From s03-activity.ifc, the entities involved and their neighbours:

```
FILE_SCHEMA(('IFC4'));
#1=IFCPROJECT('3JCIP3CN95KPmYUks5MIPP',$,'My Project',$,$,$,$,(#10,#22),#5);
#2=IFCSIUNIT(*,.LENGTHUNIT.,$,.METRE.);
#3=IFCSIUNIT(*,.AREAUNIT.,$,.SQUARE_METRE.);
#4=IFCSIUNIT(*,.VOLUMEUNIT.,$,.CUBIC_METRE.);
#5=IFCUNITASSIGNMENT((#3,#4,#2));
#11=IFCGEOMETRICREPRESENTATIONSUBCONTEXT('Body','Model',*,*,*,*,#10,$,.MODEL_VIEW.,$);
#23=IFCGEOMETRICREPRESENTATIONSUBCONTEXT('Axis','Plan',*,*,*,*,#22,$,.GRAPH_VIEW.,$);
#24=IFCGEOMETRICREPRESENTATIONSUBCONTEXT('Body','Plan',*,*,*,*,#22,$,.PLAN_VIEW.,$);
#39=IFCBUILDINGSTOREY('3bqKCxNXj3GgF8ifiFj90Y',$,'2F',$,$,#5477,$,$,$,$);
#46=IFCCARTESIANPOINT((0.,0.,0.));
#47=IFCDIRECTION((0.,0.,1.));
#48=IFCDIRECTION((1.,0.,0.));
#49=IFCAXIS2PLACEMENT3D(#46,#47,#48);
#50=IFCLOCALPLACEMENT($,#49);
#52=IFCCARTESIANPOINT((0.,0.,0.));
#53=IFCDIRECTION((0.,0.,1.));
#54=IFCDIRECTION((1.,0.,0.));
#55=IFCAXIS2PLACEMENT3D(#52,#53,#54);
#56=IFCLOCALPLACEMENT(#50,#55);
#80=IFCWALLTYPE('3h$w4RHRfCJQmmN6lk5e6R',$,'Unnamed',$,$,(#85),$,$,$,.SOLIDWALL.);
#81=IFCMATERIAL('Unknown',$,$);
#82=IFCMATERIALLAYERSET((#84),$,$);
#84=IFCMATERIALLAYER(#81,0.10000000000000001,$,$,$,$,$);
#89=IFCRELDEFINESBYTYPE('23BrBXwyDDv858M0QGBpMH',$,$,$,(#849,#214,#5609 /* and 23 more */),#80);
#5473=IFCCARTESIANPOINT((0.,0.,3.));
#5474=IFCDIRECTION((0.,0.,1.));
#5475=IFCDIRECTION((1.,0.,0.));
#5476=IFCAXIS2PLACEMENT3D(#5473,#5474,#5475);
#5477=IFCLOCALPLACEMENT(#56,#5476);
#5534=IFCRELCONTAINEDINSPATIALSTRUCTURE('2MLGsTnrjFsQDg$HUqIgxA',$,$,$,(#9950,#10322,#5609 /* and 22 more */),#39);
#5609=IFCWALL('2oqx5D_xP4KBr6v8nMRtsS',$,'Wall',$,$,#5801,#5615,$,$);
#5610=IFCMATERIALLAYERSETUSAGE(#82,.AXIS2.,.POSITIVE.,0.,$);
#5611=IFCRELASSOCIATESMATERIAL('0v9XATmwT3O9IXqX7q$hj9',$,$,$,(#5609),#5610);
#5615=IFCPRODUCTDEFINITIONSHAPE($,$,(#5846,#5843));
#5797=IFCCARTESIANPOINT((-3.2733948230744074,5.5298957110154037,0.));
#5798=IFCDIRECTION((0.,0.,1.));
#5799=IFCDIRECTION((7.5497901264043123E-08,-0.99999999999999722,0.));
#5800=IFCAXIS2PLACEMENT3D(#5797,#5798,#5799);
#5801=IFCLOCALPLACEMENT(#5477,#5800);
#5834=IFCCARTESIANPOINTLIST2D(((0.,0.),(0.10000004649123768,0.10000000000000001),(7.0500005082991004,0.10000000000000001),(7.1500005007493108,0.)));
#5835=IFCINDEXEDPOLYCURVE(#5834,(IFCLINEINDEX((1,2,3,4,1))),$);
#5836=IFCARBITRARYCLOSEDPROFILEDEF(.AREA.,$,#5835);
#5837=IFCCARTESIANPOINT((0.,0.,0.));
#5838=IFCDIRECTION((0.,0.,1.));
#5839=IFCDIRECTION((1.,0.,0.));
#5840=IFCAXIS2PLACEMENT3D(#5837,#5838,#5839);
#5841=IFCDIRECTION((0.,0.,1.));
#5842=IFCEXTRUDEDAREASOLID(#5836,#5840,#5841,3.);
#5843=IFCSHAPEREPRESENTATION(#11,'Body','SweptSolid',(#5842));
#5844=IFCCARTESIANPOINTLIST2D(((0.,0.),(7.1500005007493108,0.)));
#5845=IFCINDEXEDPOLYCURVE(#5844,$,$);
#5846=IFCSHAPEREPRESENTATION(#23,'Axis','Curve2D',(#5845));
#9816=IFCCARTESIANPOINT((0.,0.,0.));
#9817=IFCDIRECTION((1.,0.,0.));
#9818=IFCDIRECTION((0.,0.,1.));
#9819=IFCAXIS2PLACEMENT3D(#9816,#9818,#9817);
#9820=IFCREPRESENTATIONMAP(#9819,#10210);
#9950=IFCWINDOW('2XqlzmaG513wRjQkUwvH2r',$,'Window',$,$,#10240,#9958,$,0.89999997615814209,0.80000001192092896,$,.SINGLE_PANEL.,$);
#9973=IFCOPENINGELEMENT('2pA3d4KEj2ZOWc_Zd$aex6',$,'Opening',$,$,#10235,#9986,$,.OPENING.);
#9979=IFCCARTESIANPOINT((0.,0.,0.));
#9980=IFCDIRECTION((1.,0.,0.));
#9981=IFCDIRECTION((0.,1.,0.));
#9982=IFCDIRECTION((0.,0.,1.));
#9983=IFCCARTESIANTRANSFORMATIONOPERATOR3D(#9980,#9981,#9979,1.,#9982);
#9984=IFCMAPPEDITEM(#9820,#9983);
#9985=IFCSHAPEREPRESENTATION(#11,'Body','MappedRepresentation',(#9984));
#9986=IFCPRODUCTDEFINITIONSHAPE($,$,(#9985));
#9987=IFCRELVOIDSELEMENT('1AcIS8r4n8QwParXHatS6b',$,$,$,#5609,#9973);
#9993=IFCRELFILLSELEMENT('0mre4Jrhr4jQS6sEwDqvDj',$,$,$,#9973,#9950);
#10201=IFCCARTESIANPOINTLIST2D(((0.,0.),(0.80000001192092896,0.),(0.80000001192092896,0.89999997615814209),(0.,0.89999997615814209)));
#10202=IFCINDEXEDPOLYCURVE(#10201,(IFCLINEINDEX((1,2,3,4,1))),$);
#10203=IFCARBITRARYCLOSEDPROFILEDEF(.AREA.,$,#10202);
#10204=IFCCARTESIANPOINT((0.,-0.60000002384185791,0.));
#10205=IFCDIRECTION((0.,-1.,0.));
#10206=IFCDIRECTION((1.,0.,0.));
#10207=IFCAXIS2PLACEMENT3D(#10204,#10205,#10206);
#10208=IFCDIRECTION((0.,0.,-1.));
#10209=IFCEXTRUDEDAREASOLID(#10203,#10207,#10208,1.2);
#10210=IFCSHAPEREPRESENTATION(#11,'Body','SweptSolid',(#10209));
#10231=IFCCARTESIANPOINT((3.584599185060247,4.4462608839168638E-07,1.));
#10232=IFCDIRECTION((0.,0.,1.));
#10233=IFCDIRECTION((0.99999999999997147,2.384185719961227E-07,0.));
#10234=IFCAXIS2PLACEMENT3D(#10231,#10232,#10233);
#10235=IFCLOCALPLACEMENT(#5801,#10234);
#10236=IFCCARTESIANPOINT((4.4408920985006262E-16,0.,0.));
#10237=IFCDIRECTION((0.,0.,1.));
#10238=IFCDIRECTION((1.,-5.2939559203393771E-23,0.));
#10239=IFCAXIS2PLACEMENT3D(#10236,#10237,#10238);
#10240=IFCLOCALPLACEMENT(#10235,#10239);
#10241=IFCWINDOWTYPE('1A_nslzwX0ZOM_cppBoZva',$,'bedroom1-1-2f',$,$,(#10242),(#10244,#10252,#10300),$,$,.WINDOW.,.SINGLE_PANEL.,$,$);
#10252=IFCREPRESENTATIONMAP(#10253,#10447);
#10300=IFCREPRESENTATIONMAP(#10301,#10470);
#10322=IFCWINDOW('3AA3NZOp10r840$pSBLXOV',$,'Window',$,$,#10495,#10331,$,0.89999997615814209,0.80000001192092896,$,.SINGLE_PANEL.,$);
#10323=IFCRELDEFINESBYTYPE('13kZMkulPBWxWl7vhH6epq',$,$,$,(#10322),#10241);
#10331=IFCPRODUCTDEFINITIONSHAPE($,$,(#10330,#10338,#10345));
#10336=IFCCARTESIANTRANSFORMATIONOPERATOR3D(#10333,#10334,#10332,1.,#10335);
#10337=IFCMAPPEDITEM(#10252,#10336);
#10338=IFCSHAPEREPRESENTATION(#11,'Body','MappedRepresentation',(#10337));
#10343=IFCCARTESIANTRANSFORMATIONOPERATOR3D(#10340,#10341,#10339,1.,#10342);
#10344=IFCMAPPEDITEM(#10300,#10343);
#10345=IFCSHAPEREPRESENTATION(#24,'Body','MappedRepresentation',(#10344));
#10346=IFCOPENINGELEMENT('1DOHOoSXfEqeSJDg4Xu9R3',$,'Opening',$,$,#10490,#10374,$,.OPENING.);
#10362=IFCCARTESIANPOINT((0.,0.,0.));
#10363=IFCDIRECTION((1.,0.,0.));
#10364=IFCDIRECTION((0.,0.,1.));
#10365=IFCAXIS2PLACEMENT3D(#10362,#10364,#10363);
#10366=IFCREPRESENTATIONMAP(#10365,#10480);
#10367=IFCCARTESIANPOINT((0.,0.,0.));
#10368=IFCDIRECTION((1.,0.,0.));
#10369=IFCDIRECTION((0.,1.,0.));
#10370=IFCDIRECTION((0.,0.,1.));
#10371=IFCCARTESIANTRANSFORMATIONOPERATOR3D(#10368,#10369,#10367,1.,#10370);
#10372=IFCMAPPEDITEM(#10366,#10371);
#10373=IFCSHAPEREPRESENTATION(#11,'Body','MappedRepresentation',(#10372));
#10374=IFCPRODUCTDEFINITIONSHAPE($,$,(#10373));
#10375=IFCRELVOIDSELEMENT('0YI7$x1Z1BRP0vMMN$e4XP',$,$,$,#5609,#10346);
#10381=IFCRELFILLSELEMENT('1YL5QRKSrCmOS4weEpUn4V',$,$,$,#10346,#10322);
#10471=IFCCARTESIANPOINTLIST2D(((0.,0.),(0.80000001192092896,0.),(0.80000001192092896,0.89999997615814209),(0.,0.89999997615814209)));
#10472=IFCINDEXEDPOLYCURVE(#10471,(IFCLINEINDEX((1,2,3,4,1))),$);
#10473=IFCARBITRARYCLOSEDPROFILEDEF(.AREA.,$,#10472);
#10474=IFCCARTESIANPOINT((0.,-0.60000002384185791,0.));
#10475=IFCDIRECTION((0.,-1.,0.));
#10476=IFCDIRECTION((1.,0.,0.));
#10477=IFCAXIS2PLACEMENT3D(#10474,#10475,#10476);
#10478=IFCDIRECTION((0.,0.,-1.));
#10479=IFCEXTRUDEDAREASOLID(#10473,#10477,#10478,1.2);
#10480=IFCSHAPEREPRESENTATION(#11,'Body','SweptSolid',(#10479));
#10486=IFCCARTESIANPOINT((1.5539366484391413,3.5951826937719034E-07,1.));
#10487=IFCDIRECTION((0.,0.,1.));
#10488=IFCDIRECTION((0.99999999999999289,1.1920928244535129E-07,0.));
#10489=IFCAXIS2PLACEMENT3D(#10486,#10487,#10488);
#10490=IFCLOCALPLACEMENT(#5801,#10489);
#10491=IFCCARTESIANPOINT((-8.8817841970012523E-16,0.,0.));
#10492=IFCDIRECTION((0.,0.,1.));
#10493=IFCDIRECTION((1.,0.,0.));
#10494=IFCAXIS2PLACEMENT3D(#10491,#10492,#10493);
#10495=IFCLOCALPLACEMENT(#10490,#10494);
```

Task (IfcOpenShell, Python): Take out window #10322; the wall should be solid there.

```python
import ifcopenshell
import ifcopenshell.api.feature
import ifcopenshell.api.root
import ifcopenshell.geom
import ifcopenshell.util.shape

model = ifcopenshell.open("s03-activity.ifc")
settings = ifcopenshell.geom.settings()


def volume(element):
    """Net volume in cubic metres, openings subtracted."""
    shape = ifcopenshell.geom.create_shape(settings, element)
    return ifcopenshell.util.shape.get_volume(shape.geometry)


window = model.by_guid("3AA3NZOp10r840$pSBLXOV")
opening = window.FillsVoids[0].RelatingOpeningElement
wall = opening.VoidsElements[0].RelatingBuildingElement
before = volume(wall)

ifcopenshell.api.root.remove_product(model, product=window)
ifcopenshell.api.feature.remove_feature(model, feature=opening)

after = volume(wall)

print(f"wall volume {before:.3f} -> {after:.3f} m3")

model.write("s03-activity_rev.ifc")
```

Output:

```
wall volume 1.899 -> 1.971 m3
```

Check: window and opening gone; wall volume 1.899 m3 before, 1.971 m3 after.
